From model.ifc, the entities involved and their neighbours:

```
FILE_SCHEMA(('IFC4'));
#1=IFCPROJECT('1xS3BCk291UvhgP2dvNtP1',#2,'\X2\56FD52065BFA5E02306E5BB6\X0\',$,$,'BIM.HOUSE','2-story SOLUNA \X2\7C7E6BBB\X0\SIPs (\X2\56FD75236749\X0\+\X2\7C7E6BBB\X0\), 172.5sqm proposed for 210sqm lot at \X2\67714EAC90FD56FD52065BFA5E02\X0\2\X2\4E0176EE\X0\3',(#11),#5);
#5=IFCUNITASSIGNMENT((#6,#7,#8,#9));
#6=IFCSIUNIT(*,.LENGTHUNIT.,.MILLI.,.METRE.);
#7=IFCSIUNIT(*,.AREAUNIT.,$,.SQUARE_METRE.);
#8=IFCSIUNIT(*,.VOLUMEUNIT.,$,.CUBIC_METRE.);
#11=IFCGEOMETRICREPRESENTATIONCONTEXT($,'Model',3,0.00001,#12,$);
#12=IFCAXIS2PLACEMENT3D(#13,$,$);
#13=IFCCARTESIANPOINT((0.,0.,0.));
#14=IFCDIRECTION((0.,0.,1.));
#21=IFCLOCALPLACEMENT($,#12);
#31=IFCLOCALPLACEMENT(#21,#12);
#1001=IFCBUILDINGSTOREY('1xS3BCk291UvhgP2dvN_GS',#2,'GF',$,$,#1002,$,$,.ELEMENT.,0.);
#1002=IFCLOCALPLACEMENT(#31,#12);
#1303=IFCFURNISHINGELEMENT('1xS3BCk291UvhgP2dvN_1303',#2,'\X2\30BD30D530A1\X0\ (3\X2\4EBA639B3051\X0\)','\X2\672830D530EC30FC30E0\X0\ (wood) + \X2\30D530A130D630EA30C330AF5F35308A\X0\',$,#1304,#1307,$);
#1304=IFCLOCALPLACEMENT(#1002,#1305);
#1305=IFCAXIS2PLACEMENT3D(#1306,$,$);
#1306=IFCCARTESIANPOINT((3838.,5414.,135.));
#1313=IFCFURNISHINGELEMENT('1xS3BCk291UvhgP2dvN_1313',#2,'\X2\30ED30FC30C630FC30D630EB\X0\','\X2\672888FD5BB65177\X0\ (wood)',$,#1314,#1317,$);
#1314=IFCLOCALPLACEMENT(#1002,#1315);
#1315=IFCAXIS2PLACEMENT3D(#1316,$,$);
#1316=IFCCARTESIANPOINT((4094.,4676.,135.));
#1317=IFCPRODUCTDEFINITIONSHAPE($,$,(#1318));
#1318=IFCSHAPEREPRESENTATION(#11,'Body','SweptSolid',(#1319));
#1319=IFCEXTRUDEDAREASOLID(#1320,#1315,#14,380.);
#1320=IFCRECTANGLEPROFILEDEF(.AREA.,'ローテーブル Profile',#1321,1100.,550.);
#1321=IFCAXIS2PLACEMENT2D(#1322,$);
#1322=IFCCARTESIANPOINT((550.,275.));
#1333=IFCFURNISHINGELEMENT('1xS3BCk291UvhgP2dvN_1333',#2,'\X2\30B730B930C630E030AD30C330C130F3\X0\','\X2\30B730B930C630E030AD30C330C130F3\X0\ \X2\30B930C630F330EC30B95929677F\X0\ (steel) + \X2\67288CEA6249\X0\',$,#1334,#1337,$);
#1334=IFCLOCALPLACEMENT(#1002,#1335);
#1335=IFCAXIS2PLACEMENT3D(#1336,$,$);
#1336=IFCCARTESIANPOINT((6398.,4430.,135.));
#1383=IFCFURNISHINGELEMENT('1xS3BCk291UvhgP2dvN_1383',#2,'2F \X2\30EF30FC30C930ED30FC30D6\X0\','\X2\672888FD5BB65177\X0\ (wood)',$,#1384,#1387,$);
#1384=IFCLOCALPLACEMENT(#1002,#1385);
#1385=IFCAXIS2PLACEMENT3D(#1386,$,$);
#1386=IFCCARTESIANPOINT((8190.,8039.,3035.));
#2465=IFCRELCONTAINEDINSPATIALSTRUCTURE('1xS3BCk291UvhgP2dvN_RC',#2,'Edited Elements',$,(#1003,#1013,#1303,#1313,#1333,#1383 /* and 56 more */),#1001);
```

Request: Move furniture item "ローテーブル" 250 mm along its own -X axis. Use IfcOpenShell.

```python
import ifcopenshell
import ifcopenshell.api.geometry
import ifcopenshell.util.placement
import ifcopenshell.util.unit

model = ifcopenshell.open("model.ifc")
unit_scale = ifcopenshell.util.unit.calculate_unit_scale(model)

item = model.by_guid("1xS3BCk291UvhgP2dvN_1313")
matrix = ifcopenshell.util.placement.get_local_placement(item.ObjectPlacement)
matrix[:3, 3] -= matrix[:3, 0] * 0.25 / unit_scale
ifcopenshell.api.geometry.edit_object_placement(model, product=item, matrix=matrix, is_si=False)

print(ifcopenshell.util.placement.get_local_placement(item.ObjectPlacement).round(3) + 0.0)

model.write("model_v2.ifc")
```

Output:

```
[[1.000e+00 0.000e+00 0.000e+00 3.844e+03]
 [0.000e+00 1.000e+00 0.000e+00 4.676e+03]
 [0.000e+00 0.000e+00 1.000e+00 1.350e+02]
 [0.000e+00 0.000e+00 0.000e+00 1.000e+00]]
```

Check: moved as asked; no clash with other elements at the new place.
